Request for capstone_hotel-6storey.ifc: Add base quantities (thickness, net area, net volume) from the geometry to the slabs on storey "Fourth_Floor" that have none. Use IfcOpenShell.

First a look at what the model holds.

```python
import ifcopenshell
import ifcopenshell.util.element
import ifcopenshell.util.unit

model = ifcopenshell.open("capstone_hotel-6storey.ifc")
print(model.schema)
for unit_type in ("LENGTHUNIT", "AREAUNIT", "VOLUMEUNIT"):
    print(unit_type, ifcopenshell.util.unit.calculate_unit_scale(model, unit_type))
storey = next(s for s in model.by_type("IfcBuildingStorey") if s.Name == "Fourth_Floor")
slabs = [e for e in ifcopenshell.util.element.get_decomposition(storey) if e.is_a("IfcSlab")]
for e in sorted(slabs, key=lambda e: e.id()):
    print(e.id(), e.is_a(), e.Name, list(ifcopenshell.util.element.get_psets(e, qtos_only=True)), sep=" | ")
```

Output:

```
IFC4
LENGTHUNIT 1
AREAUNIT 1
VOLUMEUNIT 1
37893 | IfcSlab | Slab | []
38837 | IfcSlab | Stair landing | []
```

```python
import ifcopenshell
import ifcopenshell.api.pset
import ifcopenshell.geom
import ifcopenshell.util.element
import ifcopenshell.util.shape
import ifcopenshell.util.unit

model = ifcopenshell.open("capstone_hotel-6storey.ifc")
unit_scale = ifcopenshell.util.unit.calculate_unit_scale(model)
area_scale = ifcopenshell.util.unit.calculate_unit_scale(model, "AREAUNIT")
volume_scale = ifcopenshell.util.unit.calculate_unit_scale(model, "VOLUMEUNIT")
settings = ifcopenshell.geom.settings()

storey = next(s for s in model.by_type("IfcBuildingStorey") if s.Name == "Fourth_Floor")
slabs = [e for e in ifcopenshell.util.element.get_decomposition(storey) if e.is_a("IfcSlab")]

for e in sorted(slabs, key=lambda e: e.id()):
    if ifcopenshell.util.element.get_psets(e, qtos_only=True, should_inherit=False):
        continue
    # Geometry comes back in metres, in the element's own axes.
    shape = ifcopenshell.geom.create_shape(settings, e)
    values = {
        "Width": ifcopenshell.util.shape.get_z(shape.geometry) / unit_scale,
        "NetArea": ifcopenshell.util.shape.get_footprint_area(shape.geometry) / area_scale,
        "NetVolume": ifcopenshell.util.shape.get_volume(shape.geometry) / volume_scale,
    }
    qto = ifcopenshell.api.pset.add_qto(model, product=e, name="Qto_SlabBaseQuantities")
    ifcopenshell.api.pset.edit_qto(model, qto=qto, properties=values)
    print(e.id(), {k: round(v, 3) for k, v in values.items()})

model.write("capstone_hotel-6storey_rev.ifc")
```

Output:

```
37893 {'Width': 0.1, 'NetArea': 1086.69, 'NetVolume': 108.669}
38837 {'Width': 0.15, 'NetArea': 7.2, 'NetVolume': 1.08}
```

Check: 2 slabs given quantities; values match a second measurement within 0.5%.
